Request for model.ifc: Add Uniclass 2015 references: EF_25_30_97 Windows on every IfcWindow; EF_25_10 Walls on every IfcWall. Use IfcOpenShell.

First a look at what the model holds.

```python
import ifcopenshell

model = ifcopenshell.open("model.ifc")
print(model.schema)
print("classifications:", [c.Name for c in model.by_type("IfcClassification")])
for ifc_class in ("IfcDoor", "IfcRoof", "IfcStair", "IfcWall", "IfcWindow"):
    print(ifc_class, len(model.by_type(ifc_class)))
```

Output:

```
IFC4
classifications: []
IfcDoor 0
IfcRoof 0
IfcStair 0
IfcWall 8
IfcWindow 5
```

```python
import ifcopenshell
import ifcopenshell.api.classification

model = ifcopenshell.open("model.ifc")

system = ifcopenshell.api.classification.add_classification(model, classification="Uniclass 2015")

codes = {
    "IfcWindow": ("EF_25_30_97", "Windows"),
    "IfcWall": ("EF_25_10", "Walls"),
}
for ifc_class, (code, name) in codes.items():
    products = model.by_type(ifc_class)
    ifcopenshell.api.classification.add_reference(
        model, products=products, classification=system, identification=code, name=name
    )
    print(code, len(products))

model.write("model_v2.ifc")
```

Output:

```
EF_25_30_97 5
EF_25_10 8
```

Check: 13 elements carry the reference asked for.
